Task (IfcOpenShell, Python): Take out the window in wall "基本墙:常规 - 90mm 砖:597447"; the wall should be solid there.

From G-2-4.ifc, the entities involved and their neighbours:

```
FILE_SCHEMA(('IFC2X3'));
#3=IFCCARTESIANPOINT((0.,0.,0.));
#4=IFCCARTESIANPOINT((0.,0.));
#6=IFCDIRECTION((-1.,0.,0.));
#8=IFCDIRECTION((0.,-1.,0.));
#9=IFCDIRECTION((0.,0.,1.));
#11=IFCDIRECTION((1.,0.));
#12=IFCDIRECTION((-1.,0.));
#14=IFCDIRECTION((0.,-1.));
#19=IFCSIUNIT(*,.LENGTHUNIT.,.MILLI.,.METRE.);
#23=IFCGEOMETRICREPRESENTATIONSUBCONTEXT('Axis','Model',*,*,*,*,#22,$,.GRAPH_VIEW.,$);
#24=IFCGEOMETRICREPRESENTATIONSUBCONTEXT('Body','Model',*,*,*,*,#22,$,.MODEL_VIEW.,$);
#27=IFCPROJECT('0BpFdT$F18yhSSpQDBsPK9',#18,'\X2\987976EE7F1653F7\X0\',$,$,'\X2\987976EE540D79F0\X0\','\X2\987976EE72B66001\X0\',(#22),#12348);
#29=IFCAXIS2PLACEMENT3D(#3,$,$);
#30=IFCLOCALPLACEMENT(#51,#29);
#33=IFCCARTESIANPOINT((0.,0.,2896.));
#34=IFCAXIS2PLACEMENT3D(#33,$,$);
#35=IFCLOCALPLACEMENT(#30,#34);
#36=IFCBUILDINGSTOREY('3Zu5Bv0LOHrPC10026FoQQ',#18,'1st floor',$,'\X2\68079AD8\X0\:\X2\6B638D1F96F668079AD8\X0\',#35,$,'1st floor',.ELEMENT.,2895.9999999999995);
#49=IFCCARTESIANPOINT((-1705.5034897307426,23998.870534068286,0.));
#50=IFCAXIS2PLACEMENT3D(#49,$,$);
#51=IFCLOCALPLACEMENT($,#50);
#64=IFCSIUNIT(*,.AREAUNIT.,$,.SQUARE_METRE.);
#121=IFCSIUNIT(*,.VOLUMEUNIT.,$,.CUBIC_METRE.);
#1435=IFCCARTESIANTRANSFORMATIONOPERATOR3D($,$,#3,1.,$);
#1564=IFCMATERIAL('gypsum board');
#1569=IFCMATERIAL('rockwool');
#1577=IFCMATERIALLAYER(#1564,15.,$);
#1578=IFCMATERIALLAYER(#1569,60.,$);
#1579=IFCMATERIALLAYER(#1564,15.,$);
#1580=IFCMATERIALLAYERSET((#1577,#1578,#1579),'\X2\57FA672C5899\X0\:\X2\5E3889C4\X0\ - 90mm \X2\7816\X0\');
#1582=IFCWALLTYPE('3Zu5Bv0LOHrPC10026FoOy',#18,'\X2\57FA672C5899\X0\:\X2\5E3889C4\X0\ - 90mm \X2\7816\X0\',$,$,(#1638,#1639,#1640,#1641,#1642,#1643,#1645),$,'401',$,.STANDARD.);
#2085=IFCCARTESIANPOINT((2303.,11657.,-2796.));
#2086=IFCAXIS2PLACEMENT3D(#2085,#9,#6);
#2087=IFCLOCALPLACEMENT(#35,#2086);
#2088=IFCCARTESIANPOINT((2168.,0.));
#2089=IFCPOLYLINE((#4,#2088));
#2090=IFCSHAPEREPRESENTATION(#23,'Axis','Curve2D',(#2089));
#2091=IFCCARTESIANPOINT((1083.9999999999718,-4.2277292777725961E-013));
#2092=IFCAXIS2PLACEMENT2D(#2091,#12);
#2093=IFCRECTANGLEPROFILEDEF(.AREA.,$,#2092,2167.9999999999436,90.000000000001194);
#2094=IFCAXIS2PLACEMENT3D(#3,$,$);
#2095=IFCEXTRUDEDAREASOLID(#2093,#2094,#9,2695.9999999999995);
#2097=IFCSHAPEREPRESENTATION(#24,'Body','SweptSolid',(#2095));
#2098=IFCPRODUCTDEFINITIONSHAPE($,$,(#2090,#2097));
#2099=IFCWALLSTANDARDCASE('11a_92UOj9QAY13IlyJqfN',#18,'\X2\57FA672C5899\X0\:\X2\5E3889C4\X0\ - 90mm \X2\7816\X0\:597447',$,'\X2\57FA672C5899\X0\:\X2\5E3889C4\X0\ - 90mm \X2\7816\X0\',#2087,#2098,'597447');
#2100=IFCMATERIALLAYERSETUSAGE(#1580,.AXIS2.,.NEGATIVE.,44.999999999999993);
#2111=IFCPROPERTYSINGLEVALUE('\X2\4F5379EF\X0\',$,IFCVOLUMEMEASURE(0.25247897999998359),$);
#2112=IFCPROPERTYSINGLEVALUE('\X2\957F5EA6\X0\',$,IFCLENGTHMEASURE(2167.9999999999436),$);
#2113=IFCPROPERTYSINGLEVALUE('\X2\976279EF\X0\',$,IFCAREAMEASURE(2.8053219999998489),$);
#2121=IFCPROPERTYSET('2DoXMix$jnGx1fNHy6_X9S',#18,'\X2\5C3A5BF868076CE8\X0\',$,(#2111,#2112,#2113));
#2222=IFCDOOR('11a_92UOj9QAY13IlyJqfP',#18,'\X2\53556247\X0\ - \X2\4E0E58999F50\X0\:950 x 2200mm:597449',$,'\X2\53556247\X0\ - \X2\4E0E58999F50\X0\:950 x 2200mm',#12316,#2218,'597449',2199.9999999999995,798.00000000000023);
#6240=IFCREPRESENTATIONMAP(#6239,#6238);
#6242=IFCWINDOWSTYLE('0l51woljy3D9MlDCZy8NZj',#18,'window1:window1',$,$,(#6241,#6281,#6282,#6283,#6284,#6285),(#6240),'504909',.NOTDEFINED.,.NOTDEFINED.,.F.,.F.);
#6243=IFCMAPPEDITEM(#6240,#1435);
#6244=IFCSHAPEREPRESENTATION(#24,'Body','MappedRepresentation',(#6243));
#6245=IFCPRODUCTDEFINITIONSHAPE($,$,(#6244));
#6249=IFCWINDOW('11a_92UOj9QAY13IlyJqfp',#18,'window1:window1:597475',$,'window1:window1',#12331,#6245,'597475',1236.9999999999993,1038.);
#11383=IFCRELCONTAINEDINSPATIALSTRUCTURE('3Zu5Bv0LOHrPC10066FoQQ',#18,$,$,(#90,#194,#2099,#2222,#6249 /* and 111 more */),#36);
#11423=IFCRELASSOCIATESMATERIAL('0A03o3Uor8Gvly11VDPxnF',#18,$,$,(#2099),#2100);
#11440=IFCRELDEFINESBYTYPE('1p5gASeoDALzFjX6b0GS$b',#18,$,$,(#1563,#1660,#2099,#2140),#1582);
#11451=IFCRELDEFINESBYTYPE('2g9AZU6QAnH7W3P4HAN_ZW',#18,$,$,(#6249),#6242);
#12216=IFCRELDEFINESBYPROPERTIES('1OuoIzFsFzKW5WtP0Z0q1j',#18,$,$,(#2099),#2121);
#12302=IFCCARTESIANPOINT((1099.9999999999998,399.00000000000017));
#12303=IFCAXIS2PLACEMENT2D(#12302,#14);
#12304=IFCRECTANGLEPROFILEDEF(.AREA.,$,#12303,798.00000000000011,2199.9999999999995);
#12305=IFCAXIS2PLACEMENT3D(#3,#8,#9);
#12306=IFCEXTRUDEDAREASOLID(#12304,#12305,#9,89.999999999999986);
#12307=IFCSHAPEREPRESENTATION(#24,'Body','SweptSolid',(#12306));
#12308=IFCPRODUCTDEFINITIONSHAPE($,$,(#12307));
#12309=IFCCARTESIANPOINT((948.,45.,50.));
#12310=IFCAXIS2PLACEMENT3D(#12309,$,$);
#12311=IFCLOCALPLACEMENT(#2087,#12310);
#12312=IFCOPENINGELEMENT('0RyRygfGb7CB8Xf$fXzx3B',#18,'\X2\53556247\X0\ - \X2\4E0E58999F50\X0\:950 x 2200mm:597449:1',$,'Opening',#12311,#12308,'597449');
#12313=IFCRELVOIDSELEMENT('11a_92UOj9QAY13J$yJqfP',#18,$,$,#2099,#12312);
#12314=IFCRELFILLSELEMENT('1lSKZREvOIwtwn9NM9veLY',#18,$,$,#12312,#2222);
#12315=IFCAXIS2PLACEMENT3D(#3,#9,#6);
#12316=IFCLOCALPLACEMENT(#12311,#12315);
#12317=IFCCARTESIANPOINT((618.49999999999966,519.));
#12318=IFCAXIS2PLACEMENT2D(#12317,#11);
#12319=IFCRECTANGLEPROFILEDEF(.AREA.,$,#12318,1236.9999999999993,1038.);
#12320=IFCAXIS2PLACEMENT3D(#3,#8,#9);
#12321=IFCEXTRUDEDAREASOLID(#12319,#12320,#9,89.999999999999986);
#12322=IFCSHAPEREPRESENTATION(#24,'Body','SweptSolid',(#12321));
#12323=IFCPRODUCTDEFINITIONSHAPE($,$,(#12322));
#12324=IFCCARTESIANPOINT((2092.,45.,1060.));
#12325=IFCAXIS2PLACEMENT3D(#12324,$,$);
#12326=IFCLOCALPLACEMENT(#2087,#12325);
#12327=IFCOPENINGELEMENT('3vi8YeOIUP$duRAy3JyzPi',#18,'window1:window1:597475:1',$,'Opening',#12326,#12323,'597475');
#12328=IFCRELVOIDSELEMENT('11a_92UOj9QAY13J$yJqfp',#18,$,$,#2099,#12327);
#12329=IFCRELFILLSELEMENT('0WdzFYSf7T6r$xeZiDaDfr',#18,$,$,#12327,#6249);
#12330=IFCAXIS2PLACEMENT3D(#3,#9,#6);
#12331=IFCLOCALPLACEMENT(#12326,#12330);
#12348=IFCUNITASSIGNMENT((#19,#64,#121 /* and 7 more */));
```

```python
import ifcopenshell
import ifcopenshell.api.feature
import ifcopenshell.api.pset
import ifcopenshell.api.root
import ifcopenshell.geom
import ifcopenshell.util.element
import ifcopenshell.util.shape
import ifcopenshell.util.unit

model = ifcopenshell.open("G-2-4.ifc")
area_scale = ifcopenshell.util.unit.calculate_unit_scale(model, "AREAUNIT")
volume_scale = ifcopenshell.util.unit.calculate_unit_scale(model, "VOLUMEUNIT")
settings = ifcopenshell.geom.settings()


def volume(element):
    """Net volume in cubic metres, openings subtracted."""
    shape = ifcopenshell.geom.create_shape(settings, element)
    return ifcopenshell.util.shape.get_volume(shape.geometry)


window = model.by_guid("11a_92UOj9QAY13IlyJqfp")
opening = window.FillsVoids[0].RelatingOpeningElement
wall = opening.VoidsElements[0].RelatingBuildingElement
before = volume(wall)

ifcopenshell.api.root.remove_product(model, product=window)
ifcopenshell.api.feature.remove_feature(model, feature=opening)

after = volume(wall)
thickness = 0.09  # wall thickness in metres

# Update the wall's stored quantities.
pset = model.by_id(ifcopenshell.util.element.get_pset(wall, "尺寸标注", should_inherit=False)["id"])
ifcopenshell.api.pset.edit_pset(model, pset=pset, properties={
    "体积": model.create_entity("IfcVolumeMeasure", after / volume_scale),
    "面积": model.create_entity("IfcAreaMeasure", after / thickness / area_scale),
})

print(f"wall volume {before:.3f} -> {after:.3f} m3")

model.write("G-2-4_v2.ifc")
```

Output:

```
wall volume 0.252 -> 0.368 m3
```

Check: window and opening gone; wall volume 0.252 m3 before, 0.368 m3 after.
